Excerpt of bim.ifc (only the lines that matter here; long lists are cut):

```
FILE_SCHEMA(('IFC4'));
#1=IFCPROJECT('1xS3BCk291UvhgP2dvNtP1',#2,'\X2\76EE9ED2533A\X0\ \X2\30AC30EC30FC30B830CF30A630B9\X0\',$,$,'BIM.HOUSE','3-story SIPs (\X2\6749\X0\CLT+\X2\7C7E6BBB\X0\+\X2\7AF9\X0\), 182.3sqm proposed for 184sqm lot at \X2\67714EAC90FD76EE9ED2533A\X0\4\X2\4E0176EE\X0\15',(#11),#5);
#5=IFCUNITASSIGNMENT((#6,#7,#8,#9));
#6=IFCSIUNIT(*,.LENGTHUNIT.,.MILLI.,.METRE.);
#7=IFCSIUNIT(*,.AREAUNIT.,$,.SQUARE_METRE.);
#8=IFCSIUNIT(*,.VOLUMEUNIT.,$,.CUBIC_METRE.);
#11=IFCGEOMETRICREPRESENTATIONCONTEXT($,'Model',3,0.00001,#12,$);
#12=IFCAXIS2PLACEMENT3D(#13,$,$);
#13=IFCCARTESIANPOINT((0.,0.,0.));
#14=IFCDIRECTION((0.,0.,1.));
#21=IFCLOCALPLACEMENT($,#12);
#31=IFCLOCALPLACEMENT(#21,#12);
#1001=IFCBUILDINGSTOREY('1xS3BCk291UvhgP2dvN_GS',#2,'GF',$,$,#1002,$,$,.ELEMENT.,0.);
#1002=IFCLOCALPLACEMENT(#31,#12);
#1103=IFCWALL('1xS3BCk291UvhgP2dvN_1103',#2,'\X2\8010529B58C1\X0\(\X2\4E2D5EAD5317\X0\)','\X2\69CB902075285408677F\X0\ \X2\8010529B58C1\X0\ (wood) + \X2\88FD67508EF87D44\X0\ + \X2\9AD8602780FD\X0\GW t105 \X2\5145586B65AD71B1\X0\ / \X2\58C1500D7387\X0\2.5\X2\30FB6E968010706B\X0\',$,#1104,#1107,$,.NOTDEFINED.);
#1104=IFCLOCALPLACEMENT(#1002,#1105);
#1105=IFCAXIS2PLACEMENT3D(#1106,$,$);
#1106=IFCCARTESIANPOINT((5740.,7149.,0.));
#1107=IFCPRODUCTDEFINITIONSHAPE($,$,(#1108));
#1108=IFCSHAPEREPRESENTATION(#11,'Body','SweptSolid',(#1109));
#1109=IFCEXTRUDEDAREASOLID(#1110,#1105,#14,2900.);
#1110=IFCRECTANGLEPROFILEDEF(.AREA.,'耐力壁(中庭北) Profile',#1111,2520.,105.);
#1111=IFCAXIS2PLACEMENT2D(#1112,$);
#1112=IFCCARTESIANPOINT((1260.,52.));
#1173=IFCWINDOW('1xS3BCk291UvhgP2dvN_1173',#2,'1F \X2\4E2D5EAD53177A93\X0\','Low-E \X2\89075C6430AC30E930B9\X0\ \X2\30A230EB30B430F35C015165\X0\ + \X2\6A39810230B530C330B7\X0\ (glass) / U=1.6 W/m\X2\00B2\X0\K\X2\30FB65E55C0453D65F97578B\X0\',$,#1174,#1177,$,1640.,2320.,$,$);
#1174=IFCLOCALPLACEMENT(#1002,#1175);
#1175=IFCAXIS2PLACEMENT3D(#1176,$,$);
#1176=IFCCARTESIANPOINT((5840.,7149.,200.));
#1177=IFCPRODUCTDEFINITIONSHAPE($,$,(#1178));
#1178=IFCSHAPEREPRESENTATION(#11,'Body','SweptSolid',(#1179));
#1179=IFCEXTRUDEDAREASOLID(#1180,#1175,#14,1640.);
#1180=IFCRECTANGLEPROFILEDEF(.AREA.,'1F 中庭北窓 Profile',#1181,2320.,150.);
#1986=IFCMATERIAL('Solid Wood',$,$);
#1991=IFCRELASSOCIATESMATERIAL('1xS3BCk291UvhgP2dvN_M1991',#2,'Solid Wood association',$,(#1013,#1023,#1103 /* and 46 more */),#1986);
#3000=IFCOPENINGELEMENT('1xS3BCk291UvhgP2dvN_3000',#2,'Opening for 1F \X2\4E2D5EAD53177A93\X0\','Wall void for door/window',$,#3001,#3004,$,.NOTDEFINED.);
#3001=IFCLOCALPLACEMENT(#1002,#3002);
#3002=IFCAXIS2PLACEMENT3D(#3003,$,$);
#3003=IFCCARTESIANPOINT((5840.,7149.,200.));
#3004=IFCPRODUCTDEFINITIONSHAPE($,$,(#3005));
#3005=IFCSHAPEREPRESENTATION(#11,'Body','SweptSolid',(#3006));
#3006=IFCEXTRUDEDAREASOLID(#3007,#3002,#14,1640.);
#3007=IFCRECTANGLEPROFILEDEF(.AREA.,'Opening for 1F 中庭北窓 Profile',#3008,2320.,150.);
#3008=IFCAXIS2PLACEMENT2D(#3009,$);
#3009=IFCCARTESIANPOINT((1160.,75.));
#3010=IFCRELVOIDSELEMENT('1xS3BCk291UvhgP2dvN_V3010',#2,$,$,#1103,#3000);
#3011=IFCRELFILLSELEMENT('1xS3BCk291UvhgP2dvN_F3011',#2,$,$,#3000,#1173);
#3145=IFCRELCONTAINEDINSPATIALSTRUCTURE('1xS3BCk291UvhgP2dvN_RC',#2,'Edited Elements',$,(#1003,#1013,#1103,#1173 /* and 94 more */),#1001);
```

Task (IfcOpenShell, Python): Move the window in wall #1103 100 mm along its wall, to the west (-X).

```python
import ifcopenshell
import ifcopenshell.api.geometry
import ifcopenshell.util.placement

model = ifcopenshell.open("bim.ifc")

window = model.by_guid("1xS3BCk291UvhgP2dvN_1173")
opening = window.FillsVoids[0].RelatingOpeningElement
wall = opening.VoidsElements[0].RelatingBuildingElement

wall_matrix = ifcopenshell.util.placement.get_local_placement(wall.ObjectPlacement)
shift = wall_matrix[:3, 0] * -100.0
before = ifcopenshell.util.placement.get_local_placement(window.ObjectPlacement)[:3, 3].copy()

# The window is not placed relative to its opening, so move both.
for product in (opening, window):
    matrix = ifcopenshell.util.placement.get_local_placement(product.ObjectPlacement)
    matrix[:3, 3] += shift
    ifcopenshell.api.geometry.edit_object_placement(model, product=product, matrix=matrix, is_si=False)

after = ifcopenshell.util.placement.get_local_placement(window.ObjectPlacement)[:3, 3]
print("window moved by", (after - before).round(3) + 0.0)

model.write("bim-out.ifc")
```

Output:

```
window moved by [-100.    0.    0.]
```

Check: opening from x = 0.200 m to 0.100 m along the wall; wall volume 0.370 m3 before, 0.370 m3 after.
